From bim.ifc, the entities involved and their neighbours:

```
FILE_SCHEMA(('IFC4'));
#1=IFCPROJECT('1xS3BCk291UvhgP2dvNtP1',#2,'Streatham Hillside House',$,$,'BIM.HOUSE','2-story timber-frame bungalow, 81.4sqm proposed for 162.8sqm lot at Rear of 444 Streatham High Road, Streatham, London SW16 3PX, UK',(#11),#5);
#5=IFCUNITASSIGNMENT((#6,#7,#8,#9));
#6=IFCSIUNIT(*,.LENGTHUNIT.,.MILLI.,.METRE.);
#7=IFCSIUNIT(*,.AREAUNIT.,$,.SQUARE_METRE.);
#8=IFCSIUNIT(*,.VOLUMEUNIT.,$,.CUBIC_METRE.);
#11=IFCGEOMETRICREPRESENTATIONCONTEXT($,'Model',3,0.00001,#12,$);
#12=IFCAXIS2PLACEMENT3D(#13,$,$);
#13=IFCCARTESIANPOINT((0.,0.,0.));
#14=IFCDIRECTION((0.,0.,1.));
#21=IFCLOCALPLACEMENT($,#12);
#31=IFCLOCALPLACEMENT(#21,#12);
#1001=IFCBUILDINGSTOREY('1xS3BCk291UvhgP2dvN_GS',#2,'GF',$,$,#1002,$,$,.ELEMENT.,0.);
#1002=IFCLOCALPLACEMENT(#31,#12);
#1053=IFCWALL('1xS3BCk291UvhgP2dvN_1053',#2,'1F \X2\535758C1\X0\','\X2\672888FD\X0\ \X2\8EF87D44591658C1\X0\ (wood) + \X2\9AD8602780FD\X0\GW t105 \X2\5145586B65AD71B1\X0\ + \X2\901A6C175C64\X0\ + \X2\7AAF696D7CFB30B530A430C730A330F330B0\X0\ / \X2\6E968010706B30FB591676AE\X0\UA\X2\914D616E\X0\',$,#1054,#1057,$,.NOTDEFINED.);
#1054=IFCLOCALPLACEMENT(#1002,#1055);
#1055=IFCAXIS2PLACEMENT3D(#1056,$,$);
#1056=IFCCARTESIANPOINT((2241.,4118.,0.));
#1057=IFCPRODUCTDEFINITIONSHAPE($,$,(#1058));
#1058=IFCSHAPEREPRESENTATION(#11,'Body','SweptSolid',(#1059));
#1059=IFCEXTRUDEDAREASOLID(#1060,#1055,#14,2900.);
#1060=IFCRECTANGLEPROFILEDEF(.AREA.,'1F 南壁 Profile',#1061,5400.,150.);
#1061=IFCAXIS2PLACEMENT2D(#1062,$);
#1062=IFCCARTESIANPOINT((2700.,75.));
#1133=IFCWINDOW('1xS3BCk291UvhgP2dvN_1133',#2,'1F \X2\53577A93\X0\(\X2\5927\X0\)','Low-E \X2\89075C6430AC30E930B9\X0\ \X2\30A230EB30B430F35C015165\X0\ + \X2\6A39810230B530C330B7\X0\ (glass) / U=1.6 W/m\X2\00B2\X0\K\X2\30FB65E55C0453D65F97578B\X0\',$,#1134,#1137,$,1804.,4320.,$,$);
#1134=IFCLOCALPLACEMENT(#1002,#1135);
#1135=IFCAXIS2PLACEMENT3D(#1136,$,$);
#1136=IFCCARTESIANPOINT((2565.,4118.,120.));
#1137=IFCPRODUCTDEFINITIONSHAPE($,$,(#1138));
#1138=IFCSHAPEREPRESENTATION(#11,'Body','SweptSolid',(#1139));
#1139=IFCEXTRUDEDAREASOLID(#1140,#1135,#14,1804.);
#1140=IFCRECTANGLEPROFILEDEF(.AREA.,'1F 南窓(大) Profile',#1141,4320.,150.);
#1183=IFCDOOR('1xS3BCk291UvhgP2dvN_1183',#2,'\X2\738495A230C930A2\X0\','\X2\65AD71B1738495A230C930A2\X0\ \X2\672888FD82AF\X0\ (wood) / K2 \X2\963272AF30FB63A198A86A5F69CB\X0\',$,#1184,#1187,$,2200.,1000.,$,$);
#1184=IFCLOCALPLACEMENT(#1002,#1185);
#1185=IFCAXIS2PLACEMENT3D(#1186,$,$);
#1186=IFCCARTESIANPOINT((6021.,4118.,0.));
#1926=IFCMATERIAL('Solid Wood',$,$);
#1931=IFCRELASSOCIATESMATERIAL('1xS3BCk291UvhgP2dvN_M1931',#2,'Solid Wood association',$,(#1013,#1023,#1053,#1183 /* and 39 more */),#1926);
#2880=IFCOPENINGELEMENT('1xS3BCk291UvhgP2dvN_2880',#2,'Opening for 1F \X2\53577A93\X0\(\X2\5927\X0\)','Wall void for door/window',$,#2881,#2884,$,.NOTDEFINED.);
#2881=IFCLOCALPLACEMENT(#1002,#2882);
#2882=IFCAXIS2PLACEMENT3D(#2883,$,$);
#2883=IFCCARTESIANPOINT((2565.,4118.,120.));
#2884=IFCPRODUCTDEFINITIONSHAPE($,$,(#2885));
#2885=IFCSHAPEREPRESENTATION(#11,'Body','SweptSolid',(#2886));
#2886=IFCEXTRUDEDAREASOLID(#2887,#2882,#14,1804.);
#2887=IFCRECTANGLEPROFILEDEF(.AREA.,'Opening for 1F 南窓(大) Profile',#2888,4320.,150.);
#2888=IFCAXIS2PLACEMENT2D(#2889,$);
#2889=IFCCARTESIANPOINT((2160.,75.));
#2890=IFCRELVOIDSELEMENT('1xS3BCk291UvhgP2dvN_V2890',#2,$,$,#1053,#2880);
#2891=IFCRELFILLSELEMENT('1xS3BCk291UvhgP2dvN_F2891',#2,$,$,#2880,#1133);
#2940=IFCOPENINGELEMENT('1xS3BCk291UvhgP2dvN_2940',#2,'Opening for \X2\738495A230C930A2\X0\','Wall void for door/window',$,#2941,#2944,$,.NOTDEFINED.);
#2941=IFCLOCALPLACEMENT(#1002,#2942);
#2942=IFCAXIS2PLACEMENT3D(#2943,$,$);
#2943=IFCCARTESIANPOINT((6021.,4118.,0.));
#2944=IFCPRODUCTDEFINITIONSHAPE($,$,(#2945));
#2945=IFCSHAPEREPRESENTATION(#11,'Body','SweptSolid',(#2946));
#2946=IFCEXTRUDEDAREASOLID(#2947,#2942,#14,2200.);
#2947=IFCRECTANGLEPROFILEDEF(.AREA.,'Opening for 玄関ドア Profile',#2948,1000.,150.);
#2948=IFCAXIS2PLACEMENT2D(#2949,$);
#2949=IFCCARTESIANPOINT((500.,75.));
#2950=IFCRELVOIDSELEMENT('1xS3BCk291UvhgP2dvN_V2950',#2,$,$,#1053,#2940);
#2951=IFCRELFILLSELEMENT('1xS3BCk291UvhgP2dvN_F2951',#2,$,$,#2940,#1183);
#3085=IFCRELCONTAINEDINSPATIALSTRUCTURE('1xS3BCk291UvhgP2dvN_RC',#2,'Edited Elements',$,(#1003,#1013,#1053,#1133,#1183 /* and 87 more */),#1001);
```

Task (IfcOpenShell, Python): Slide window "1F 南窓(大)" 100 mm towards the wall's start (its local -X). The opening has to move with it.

```python
import ifcopenshell
import ifcopenshell.api.geometry
import ifcopenshell.util.placement

model = ifcopenshell.open("bim.ifc")

window = model.by_guid("1xS3BCk291UvhgP2dvN_1133")
opening = window.FillsVoids[0].RelatingOpeningElement
wall = opening.VoidsElements[0].RelatingBuildingElement

wall_matrix = ifcopenshell.util.placement.get_local_placement(wall.ObjectPlacement)
shift = wall_matrix[:3, 0] * -100.0
before = ifcopenshell.util.placement.get_local_placement(window.ObjectPlacement)[:3, 3].copy()

# The window is not placed relative to its opening, so move both.
for product in (opening, window):
    matrix = ifcopenshell.util.placement.get_local_placement(product.ObjectPlacement)
    matrix[:3, 3] += shift
    ifcopenshell.api.geometry.edit_object_placement(model, product=product, matrix=matrix, is_si=False)

after = ifcopenshell.util.placement.get_local_placement(window.ObjectPlacement)[:3, 3]
print("window moved by", (after - before).round(3) + 0.0)

model.write("bim_v2.ifc")
```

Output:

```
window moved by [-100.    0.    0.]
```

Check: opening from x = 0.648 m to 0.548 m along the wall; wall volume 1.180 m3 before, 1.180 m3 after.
